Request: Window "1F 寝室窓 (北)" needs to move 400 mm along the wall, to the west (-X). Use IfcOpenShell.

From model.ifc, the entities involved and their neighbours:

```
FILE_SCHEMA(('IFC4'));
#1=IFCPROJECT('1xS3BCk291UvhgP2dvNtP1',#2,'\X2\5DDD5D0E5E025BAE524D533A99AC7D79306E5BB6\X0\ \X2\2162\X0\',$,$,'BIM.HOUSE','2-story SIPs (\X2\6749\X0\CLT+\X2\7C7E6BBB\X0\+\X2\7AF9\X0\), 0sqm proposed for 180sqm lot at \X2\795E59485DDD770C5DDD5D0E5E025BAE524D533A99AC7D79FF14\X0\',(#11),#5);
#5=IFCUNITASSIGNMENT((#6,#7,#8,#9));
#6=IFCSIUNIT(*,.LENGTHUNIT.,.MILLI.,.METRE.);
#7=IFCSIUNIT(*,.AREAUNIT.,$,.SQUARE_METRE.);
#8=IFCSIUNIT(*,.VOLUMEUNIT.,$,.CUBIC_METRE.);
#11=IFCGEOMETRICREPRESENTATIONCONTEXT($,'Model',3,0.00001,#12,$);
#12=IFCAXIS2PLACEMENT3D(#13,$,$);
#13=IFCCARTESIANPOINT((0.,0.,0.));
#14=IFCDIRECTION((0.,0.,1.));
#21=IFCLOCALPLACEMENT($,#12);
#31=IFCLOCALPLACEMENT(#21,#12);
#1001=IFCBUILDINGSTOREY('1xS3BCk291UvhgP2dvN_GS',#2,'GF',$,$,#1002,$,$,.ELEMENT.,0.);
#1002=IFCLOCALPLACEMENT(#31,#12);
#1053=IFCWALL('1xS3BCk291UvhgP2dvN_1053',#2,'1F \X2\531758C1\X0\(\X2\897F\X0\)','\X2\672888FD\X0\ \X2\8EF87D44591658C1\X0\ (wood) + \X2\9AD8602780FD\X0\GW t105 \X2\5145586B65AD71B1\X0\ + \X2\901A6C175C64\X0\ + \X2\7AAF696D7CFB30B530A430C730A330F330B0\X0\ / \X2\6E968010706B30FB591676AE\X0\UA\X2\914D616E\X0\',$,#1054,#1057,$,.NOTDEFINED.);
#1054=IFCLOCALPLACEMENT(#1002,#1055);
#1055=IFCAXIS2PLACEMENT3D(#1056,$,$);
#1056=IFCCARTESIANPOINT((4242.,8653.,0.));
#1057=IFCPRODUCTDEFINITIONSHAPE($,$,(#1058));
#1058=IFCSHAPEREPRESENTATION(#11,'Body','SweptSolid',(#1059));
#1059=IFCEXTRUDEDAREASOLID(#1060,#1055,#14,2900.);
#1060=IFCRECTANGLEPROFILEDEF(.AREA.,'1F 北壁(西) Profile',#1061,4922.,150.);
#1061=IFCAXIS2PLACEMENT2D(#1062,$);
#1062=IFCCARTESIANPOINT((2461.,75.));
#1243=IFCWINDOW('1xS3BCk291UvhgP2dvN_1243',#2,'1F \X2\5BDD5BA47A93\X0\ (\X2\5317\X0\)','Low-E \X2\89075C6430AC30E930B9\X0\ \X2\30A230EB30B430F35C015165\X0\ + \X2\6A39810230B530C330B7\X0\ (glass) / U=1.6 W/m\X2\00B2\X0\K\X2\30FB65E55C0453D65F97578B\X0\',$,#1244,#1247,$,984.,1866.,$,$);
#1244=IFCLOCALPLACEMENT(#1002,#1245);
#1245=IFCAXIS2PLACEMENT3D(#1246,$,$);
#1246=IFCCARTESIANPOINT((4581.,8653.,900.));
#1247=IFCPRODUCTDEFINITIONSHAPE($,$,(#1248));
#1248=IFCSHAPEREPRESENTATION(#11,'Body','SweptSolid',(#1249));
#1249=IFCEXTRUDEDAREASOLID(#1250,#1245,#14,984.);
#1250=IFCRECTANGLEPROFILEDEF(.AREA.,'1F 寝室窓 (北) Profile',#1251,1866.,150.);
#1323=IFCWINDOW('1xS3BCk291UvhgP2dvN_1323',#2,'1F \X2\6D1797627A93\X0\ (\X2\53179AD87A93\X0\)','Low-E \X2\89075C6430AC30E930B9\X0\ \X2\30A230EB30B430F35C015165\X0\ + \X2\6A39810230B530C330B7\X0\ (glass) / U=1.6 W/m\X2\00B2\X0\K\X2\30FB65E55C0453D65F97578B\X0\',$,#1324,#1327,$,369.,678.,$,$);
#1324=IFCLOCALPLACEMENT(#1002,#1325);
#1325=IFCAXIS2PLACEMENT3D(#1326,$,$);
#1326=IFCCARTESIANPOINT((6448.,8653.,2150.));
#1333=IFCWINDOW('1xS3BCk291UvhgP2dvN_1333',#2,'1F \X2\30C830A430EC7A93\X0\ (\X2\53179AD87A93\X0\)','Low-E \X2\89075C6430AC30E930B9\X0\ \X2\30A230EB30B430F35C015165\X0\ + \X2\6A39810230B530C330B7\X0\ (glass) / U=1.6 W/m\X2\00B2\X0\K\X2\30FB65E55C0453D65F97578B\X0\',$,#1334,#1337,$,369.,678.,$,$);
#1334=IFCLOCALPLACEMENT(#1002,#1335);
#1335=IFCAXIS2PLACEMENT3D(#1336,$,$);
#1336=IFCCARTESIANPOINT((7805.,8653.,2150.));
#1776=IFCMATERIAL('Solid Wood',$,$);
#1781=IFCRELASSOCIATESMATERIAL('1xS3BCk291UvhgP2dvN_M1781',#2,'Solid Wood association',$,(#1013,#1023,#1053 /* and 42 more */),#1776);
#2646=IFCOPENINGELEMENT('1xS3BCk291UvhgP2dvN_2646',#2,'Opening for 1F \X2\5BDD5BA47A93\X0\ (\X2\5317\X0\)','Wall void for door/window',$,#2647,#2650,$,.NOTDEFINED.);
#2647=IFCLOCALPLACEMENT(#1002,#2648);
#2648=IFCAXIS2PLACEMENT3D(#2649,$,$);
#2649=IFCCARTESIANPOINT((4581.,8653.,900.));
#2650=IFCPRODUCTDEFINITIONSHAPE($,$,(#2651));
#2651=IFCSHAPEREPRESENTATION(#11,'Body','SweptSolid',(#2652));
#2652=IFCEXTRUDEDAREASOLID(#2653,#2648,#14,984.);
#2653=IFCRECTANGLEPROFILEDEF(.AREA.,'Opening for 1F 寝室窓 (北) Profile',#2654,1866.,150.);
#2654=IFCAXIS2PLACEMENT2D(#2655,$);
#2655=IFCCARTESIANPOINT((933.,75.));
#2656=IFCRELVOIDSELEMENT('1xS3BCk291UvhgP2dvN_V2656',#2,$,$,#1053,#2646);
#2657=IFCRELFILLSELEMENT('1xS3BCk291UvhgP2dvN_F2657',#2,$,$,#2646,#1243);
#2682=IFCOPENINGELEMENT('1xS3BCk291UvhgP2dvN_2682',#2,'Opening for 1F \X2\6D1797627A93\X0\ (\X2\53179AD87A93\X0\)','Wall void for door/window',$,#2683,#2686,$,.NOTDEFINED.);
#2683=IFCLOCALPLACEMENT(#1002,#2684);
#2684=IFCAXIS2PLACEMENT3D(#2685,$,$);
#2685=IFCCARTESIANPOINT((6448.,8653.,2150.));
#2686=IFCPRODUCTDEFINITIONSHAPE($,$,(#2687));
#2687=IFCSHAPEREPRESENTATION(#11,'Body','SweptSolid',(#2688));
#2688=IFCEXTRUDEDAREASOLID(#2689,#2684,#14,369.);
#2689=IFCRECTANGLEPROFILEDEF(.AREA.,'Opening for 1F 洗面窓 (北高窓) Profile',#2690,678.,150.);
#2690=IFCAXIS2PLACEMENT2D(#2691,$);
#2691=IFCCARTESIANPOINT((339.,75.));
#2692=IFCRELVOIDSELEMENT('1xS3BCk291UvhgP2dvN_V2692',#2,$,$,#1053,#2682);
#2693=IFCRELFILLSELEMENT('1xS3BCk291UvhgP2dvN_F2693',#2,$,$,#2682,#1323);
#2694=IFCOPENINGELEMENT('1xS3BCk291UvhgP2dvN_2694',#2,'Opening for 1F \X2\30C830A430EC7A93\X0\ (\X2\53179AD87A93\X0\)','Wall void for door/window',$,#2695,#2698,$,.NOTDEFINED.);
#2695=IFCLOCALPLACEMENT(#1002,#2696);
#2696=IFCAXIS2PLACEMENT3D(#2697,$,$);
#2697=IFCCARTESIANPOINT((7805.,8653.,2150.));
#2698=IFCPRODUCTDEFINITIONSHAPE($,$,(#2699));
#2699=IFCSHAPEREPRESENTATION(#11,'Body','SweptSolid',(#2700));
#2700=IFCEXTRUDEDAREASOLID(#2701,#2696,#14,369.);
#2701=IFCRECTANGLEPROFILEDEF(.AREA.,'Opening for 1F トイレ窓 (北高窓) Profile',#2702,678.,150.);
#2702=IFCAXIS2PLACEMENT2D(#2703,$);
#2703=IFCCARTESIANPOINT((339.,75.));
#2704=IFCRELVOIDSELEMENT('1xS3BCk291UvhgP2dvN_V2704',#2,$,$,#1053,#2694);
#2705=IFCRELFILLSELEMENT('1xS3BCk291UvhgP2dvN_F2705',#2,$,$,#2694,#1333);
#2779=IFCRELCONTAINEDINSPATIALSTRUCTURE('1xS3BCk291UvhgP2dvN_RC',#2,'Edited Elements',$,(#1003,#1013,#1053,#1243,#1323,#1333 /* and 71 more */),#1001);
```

```python
import ifcopenshell
import ifcopenshell.api.geometry
import ifcopenshell.util.placement

model = ifcopenshell.open("model.ifc")

window = model.by_guid("1xS3BCk291UvhgP2dvN_1243")
opening = window.FillsVoids[0].RelatingOpeningElement
wall = opening.VoidsElements[0].RelatingBuildingElement

wall_matrix = ifcopenshell.util.placement.get_local_placement(wall.ObjectPlacement)
shift = wall_matrix[:3, 0] * -400.0
before = ifcopenshell.util.placement.get_local_placement(window.ObjectPlacement)[:3, 3].copy()

# The window is not placed relative to its opening, so move both.
for product in (opening, window):
    matrix = ifcopenshell.util.placement.get_local_placement(product.ObjectPlacement)
    matrix[:3, 3] += shift
    ifcopenshell.api.geometry.edit_object_placement(model, product=product, matrix=matrix, is_si=False)

after = ifcopenshell.util.placement.get_local_placement(window.ObjectPlacement)[:3, 3]
print("window moved by", (after - before).round(3) + 0.0)

model.write("model_v2.ifc")
```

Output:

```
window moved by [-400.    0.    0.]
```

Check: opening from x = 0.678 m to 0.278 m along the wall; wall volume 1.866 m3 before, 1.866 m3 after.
